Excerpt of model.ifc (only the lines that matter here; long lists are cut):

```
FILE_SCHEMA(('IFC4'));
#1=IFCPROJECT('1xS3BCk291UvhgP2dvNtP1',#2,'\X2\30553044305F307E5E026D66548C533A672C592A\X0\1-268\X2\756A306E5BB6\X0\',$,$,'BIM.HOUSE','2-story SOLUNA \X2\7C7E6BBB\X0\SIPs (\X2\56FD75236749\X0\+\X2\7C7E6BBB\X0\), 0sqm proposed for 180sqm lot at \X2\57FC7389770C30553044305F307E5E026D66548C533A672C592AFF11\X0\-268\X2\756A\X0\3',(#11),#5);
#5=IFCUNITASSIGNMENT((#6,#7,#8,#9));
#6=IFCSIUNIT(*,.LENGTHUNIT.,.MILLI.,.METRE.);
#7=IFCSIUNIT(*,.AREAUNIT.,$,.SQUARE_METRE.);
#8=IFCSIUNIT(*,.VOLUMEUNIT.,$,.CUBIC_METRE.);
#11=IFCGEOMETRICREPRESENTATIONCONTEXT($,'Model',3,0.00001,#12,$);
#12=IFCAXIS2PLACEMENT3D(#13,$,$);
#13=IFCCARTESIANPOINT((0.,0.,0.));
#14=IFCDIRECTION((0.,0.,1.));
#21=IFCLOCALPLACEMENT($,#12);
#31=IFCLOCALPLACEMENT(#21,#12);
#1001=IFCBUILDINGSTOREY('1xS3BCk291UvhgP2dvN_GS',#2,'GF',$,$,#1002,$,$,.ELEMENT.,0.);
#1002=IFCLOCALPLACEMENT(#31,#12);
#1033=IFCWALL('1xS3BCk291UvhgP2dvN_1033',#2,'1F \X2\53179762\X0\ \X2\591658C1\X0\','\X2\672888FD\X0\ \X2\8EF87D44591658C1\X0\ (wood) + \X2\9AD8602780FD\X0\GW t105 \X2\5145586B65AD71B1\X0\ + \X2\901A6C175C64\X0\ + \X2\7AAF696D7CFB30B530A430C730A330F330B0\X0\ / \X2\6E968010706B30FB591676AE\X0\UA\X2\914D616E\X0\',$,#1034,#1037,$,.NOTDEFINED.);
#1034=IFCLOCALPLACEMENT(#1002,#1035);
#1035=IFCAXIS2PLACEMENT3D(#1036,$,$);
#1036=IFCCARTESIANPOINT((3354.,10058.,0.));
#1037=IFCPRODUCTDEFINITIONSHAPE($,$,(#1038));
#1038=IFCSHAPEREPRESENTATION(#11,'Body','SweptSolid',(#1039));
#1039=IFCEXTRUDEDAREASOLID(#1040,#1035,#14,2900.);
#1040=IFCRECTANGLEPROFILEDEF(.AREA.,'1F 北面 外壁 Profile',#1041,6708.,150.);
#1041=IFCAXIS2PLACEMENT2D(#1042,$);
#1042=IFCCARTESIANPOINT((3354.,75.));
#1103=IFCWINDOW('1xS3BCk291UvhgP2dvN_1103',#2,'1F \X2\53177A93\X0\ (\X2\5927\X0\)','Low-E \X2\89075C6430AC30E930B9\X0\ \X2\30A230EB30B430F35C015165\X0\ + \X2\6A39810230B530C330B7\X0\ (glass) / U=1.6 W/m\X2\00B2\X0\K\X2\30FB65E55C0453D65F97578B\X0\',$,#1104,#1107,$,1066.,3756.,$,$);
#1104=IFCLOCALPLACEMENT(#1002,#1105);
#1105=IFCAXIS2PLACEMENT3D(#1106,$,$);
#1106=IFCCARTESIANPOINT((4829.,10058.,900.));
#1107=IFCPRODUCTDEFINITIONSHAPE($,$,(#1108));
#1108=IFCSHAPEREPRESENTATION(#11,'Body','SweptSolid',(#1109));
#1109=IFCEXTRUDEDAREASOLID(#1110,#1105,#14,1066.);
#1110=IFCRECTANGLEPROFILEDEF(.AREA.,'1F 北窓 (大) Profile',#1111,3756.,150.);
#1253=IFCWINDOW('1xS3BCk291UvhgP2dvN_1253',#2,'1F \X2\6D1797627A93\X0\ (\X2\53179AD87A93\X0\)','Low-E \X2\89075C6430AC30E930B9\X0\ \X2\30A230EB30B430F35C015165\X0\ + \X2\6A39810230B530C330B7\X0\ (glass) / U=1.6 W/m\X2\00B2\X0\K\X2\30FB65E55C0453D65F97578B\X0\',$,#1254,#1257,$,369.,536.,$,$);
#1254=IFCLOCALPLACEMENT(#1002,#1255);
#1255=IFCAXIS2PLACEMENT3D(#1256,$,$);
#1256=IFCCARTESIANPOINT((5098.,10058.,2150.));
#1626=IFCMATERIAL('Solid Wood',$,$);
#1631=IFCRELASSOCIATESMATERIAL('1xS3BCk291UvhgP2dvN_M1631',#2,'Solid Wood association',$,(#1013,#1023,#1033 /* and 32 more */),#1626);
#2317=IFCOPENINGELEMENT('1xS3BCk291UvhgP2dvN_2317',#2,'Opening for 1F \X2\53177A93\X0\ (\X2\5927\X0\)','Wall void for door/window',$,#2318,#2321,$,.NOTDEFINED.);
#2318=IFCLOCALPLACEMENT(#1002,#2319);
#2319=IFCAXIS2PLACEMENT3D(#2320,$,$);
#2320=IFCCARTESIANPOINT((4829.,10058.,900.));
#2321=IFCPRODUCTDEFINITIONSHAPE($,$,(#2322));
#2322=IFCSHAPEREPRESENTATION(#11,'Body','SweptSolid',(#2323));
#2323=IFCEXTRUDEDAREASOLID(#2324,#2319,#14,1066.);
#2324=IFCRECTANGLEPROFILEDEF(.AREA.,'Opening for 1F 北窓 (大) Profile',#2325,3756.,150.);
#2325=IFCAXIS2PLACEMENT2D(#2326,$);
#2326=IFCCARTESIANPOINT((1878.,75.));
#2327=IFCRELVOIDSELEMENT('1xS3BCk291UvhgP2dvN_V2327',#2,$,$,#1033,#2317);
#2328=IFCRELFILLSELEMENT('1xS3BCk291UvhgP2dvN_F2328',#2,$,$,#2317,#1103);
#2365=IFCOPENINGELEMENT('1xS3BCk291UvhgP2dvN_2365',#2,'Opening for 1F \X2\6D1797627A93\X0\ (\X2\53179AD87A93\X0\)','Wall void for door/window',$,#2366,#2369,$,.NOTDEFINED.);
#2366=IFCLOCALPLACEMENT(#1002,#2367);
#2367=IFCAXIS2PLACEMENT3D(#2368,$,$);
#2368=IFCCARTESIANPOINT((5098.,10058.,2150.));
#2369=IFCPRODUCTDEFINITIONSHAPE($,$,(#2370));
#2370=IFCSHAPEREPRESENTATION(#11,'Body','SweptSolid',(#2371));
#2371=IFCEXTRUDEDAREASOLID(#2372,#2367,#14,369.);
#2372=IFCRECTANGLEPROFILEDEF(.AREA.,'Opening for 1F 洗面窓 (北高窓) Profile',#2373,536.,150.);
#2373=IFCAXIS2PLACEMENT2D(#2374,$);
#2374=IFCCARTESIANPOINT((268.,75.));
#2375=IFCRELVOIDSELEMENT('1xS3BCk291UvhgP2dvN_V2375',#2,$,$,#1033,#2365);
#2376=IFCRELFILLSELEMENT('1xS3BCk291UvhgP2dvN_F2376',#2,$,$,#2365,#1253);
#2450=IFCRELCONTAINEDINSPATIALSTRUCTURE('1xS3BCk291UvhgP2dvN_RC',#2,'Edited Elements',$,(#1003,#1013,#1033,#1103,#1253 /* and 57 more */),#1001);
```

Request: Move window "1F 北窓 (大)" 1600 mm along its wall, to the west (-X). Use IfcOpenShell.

```python
import ifcopenshell
import ifcopenshell.api.geometry
import ifcopenshell.util.placement
import ifcopenshell.util.unit

model = ifcopenshell.open("model.ifc")
unit_scale = ifcopenshell.util.unit.calculate_unit_scale(model)

window = model.by_guid("1xS3BCk291UvhgP2dvN_1103")
opening = window.FillsVoids[0].RelatingOpeningElement
wall = opening.VoidsElements[0].RelatingBuildingElement

wall_matrix = ifcopenshell.util.placement.get_local_placement(wall.ObjectPlacement)
shift = wall_matrix[:3, 0] * -1.6 / unit_scale
before = ifcopenshell.util.placement.get_local_placement(window.ObjectPlacement)[:3, 3].copy()

# The window is not placed relative to its opening, so move both.
for product in (opening, window):
    matrix = ifcopenshell.util.placement.get_local_placement(product.ObjectPlacement)
    matrix[:3, 3] += shift
    ifcopenshell.api.geometry.edit_object_placement(model, product=product, matrix=matrix, is_si=False)

after = ifcopenshell.util.placement.get_local_placement(window.ObjectPlacement)[:3, 3]
print("window moved by", (after - before).round(3) + 0.0)

model.write("model-out.ifc")
```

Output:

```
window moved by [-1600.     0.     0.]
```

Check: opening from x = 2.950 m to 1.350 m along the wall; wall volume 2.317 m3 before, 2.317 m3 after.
